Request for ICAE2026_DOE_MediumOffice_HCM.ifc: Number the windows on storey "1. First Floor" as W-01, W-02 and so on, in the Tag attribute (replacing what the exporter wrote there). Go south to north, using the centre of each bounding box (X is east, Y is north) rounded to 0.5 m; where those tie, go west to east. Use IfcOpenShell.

First a look at what the model holds.

```python
import ifcopenshell
import ifcopenshell.util.element
import ifcopenshell.util.placement

model = ifcopenshell.open("ICAE2026_DOE_MediumOffice_HCM.ifc")
print(model.schema)
storey = next(s for s in model.by_type("IfcBuildingStorey") if s.Name == "1. First Floor")
windows = [e for e in ifcopenshell.util.element.get_decomposition(storey) if e.is_a("IfcWindow")]
for e in sorted(windows, key=lambda e: e.id()):
    origin = ifcopenshell.util.placement.get_local_placement(e.ObjectPlacement)[:3, 3]
    print(e.id(), e.Tag, e.Name, origin.round(2) + 0.0, sep=" | ")
```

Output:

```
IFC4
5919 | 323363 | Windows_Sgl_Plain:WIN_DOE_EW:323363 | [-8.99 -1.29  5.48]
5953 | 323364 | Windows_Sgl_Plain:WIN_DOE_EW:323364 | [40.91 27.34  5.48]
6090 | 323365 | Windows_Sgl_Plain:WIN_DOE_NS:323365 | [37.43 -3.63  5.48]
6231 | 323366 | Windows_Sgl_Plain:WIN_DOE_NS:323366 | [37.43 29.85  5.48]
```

```python
import ifcopenshell
import ifcopenshell.geom
import ifcopenshell.util.element
import ifcopenshell.util.shape

model = ifcopenshell.open("ICAE2026_DOE_MediumOffice_HCM.ifc")
settings = ifcopenshell.geom.settings()
settings.set("use-world-coords", True)


def centre(element):
    shape = ifcopenshell.geom.create_shape(settings, element)
    return ifcopenshell.util.shape.get_bbox_centroid(shape.geometry)


storey = next(s for s in model.by_type("IfcBuildingStorey") if s.Name == "1. First Floor")
windows = [e for e in ifcopenshell.util.element.get_decomposition(storey) if e.is_a("IfcWindow")]

# Insertion points can sit at a corner or the storey origin, so sort by the geometry (in metres).
centres = {e: centre(e) for e in windows}
windows.sort(key=lambda e: (round(centres[e][1] / 0.5), centres[e][0]))

for i, e in enumerate(windows, start=1):
    number = f"W-{i:02d}"
    e.Tag = number
    print(e.id(), number)

model.write("ICAE2026_DOE_MediumOffice_HCM-out.ifc")
```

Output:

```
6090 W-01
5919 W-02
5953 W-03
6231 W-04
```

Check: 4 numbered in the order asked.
